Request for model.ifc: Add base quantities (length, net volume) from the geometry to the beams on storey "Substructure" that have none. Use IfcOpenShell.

First a look at what the model holds.

```python
import ifcopenshell
import ifcopenshell.util.element
import ifcopenshell.util.unit

model = ifcopenshell.open("model.ifc")
print(model.schema)
for unit_type in ("LENGTHUNIT", "AREAUNIT", "VOLUMEUNIT"):
    print(unit_type, ifcopenshell.util.unit.calculate_unit_scale(model, unit_type))
storey = next(s for s in model.by_type("IfcBuildingStorey") if s.Name == "Substructure")
beams = [e for e in ifcopenshell.util.element.get_decomposition(storey) if e.is_a("IfcBeam")]
for e in sorted(beams, key=lambda e: e.id()):
    print(e.id(), e.is_a(), e.Name, list(ifcopenshell.util.element.get_psets(e, qtos_only=True)), sep=" | ")
```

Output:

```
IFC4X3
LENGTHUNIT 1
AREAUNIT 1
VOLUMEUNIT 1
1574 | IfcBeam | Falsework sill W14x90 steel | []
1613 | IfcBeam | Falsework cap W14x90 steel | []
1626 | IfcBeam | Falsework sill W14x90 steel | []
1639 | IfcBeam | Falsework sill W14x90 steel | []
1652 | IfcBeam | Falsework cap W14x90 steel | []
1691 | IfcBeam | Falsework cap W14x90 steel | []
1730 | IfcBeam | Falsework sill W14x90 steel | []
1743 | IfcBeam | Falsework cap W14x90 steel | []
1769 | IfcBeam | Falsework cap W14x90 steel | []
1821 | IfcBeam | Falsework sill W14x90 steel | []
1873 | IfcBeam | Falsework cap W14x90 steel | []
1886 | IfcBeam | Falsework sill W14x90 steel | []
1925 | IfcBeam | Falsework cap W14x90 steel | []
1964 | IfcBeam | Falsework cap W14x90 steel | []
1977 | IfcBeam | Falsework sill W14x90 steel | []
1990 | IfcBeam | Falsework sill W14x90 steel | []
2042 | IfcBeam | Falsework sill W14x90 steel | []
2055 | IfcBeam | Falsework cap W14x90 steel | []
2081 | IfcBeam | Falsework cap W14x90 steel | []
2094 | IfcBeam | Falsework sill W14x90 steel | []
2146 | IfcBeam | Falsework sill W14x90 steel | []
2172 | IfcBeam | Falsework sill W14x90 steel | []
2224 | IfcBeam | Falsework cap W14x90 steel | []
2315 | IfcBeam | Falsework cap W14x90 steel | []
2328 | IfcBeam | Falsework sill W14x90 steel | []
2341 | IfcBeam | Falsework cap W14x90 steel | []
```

```python
import ifcopenshell
import ifcopenshell.api.pset
import ifcopenshell.geom
import ifcopenshell.util.element
import ifcopenshell.util.shape
import ifcopenshell.util.unit

model = ifcopenshell.open("model.ifc")
unit_scale = ifcopenshell.util.unit.calculate_unit_scale(model)
volume_scale = ifcopenshell.util.unit.calculate_unit_scale(model, "VOLUMEUNIT")
settings = ifcopenshell.geom.settings()

storey = next(s for s in model.by_type("IfcBuildingStorey") if s.Name == "Substructure")
beams = [e for e in ifcopenshell.util.element.get_decomposition(storey) if e.is_a("IfcBeam")]

for e in sorted(beams, key=lambda e: e.id()):
    if ifcopenshell.util.element.get_psets(e, qtos_only=True, should_inherit=False):
        continue
    # Geometry comes back in metres, in the element's own axes.
    shape = ifcopenshell.geom.create_shape(settings, e)
    values = {
        "Length": ifcopenshell.util.shape.get_max_xyz(shape.geometry) / unit_scale,
        "NetVolume": ifcopenshell.util.shape.get_volume(shape.geometry) / volume_scale,
    }
    qto = ifcopenshell.api.pset.add_qto(model, product=e, name="Qto_BeamBaseQuantities")
    ifcopenshell.api.pset.edit_qto(model, qto=qto, properties=values)
    print(e.id(), {k: round(v, 3) for k, v in values.items()})

model.write("model_updated.ifc")
```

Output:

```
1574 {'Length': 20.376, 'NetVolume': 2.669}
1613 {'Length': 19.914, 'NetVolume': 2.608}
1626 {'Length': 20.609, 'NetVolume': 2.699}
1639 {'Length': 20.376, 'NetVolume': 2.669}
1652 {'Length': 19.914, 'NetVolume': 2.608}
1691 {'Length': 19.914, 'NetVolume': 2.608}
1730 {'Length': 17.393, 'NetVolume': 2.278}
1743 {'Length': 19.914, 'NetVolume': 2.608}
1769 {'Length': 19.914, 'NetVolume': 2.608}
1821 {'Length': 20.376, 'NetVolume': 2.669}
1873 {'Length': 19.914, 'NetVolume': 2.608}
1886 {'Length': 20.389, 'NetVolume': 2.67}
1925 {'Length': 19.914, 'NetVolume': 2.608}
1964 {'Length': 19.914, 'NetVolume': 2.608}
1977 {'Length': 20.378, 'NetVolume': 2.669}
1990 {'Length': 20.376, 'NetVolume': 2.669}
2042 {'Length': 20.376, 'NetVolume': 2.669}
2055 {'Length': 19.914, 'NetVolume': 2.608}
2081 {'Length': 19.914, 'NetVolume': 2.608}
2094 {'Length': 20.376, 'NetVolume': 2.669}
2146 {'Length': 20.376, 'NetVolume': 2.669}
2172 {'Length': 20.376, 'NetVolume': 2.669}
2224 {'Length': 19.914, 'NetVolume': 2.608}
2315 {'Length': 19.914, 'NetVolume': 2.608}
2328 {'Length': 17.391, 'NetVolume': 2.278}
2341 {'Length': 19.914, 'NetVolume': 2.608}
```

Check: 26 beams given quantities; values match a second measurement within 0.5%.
